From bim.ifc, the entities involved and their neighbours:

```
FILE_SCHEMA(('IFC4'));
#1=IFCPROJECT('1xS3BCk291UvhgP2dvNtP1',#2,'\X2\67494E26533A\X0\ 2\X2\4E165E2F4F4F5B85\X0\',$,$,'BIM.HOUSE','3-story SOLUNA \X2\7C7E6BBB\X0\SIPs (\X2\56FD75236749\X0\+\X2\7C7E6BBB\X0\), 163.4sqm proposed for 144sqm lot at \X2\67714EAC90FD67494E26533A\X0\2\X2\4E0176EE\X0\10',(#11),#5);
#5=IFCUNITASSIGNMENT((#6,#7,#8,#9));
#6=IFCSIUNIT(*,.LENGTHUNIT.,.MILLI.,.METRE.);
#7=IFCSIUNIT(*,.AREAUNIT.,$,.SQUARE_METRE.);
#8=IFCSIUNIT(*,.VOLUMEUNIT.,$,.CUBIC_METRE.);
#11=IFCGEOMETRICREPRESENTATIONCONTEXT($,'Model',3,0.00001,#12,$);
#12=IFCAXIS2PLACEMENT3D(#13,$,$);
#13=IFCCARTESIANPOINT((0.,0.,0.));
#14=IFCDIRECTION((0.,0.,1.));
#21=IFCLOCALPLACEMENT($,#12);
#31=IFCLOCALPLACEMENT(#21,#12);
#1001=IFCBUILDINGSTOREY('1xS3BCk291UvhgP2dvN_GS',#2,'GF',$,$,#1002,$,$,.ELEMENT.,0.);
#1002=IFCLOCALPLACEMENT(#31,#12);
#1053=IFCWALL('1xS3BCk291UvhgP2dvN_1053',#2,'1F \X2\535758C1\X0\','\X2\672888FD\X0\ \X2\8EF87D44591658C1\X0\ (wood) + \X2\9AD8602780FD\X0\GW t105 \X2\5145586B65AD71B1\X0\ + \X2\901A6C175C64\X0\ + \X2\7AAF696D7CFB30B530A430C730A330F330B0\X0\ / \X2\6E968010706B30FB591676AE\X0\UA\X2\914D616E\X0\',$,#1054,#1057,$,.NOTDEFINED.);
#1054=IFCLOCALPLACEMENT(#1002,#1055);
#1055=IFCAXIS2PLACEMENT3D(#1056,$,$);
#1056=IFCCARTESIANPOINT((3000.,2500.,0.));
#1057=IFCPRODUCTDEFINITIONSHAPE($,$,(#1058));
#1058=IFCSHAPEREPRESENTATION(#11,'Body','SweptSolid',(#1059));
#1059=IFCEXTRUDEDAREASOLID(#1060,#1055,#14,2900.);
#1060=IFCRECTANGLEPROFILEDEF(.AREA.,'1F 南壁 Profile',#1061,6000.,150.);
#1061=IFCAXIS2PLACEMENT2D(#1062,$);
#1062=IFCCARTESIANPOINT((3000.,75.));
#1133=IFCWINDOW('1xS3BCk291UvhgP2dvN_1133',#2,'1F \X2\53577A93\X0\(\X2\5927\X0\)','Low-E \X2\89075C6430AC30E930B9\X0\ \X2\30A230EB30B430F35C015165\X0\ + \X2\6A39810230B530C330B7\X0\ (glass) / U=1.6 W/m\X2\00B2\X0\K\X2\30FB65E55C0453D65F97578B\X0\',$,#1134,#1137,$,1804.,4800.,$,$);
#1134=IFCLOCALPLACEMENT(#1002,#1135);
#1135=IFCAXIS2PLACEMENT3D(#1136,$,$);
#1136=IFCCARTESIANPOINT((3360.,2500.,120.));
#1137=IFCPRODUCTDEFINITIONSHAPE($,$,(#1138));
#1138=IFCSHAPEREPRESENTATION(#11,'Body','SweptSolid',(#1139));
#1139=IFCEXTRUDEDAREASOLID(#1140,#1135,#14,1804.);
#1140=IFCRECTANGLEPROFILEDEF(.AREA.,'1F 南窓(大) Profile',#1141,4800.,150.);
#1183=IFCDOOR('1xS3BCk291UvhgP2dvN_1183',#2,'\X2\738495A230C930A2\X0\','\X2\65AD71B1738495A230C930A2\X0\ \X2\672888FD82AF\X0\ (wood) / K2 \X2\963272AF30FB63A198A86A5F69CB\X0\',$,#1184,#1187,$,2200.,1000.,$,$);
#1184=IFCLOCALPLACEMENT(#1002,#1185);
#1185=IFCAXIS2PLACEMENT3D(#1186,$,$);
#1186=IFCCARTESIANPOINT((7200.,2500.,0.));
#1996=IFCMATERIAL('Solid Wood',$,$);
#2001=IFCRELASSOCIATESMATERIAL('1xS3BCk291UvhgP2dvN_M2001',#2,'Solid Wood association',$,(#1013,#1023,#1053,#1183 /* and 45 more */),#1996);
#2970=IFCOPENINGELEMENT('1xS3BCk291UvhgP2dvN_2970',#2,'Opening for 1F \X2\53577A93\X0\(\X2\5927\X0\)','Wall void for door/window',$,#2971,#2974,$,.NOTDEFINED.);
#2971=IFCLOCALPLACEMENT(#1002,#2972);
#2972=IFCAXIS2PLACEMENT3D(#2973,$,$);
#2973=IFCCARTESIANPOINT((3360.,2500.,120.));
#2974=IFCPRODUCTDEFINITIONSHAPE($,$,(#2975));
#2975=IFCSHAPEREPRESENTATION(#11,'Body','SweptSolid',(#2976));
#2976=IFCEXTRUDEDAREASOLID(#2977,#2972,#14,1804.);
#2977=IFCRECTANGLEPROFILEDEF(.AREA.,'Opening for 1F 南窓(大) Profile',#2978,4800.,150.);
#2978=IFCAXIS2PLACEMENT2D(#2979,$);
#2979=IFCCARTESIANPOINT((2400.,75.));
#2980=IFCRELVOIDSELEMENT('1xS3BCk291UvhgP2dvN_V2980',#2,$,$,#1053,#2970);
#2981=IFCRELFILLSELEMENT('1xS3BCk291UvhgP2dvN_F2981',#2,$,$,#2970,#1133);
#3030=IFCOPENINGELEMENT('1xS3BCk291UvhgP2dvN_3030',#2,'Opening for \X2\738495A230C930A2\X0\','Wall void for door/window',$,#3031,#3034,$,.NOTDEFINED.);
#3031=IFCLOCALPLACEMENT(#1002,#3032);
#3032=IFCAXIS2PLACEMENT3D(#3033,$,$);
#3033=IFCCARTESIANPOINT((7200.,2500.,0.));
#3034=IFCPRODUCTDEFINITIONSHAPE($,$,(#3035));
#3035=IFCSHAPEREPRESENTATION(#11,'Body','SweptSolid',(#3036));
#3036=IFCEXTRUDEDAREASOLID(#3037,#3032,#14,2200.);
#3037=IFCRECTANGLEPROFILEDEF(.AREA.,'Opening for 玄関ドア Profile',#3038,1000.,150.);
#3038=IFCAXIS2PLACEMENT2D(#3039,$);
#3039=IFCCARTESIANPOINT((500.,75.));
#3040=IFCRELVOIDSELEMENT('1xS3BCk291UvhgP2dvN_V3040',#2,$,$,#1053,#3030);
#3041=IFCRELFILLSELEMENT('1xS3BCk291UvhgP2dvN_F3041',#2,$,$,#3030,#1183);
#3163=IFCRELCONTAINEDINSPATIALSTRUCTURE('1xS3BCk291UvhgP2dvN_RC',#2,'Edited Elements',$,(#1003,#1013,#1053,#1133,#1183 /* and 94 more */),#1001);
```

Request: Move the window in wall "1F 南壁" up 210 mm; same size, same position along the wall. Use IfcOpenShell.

```python
import numpy as np
import ifcopenshell
import ifcopenshell.api.geometry
import ifcopenshell.util.placement
import ifcopenshell.util.unit

model = ifcopenshell.open("bim.ifc")
unit_scale = ifcopenshell.util.unit.calculate_unit_scale(model)

window = model.by_guid("1xS3BCk291UvhgP2dvN_1133")
opening = window.FillsVoids[0].RelatingOpeningElement
dz = 210.0

shift = np.array([0.0, 0.0, dz])
# The window is not placed relative to its opening, so move both.
for product in (opening, window):
    matrix = ifcopenshell.util.placement.get_local_placement(product.ObjectPlacement)
    matrix[:3, 3] += shift
    ifcopenshell.api.geometry.edit_object_placement(model, product=product, matrix=matrix, is_si=False)

print(f"moved by {dz * unit_scale:+.3f} m")

model.write("bim_edited.ifc")
```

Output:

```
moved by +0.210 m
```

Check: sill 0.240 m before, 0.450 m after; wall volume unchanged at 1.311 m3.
